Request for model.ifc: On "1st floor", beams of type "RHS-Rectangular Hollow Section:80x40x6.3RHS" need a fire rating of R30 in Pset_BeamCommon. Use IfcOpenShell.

First a look at what the model holds.

```python
import ifcopenshell
import ifcopenshell.util.element

model = ifcopenshell.open("model.ifc")
print(model.schema)
storey = next(s for s in model.by_type("IfcBuildingStorey") if s.Name == "1st floor")
beams = [e for e in ifcopenshell.util.element.get_decomposition(storey) if e.is_a("IfcBeam")]
seen = {}
for e in beams:
    element_type = ifcopenshell.util.element.get_type(e)
    key = (element_type.Name if element_type != e and element_type else None, ifcopenshell.util.element.get_pset(e, "Pset_BeamCommon", "FireRating"))
    seen[key] = seen.get(key, 0) + 1
for (name, value), count in sorted(seen.items(), key=str):
    print(count, "x", name, "|", value)
```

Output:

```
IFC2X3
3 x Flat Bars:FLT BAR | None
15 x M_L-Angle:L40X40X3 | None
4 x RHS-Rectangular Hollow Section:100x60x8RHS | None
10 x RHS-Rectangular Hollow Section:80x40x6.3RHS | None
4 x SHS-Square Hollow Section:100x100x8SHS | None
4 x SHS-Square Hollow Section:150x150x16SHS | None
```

```python
import ifcopenshell
import ifcopenshell.api.pset
import ifcopenshell.util.element

model = ifcopenshell.open("model.ifc")

storey = next(s for s in model.by_type("IfcBuildingStorey") if s.Name == "1st floor")
beams = [e for e in ifcopenshell.util.element.get_decomposition(storey) if e.is_a("IfcBeam")]

count = 0
for e in beams:
    element_type = ifcopenshell.util.element.get_type(e)
    if element_type in (None, e) or element_type.Name != "RHS-Rectangular Hollow Section:80x40x6.3RHS":
        continue
    # add_pset returns the element's existing set when there is one.
    pset = ifcopenshell.api.pset.add_pset(model, product=e, name="Pset_BeamCommon")
    ifcopenshell.api.pset.edit_pset(model, pset=pset, properties={"FireRating": "R30"})
    count += 1

print(count, "beams updated")

model.write("model-out.ifc")
```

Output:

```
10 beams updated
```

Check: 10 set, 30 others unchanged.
